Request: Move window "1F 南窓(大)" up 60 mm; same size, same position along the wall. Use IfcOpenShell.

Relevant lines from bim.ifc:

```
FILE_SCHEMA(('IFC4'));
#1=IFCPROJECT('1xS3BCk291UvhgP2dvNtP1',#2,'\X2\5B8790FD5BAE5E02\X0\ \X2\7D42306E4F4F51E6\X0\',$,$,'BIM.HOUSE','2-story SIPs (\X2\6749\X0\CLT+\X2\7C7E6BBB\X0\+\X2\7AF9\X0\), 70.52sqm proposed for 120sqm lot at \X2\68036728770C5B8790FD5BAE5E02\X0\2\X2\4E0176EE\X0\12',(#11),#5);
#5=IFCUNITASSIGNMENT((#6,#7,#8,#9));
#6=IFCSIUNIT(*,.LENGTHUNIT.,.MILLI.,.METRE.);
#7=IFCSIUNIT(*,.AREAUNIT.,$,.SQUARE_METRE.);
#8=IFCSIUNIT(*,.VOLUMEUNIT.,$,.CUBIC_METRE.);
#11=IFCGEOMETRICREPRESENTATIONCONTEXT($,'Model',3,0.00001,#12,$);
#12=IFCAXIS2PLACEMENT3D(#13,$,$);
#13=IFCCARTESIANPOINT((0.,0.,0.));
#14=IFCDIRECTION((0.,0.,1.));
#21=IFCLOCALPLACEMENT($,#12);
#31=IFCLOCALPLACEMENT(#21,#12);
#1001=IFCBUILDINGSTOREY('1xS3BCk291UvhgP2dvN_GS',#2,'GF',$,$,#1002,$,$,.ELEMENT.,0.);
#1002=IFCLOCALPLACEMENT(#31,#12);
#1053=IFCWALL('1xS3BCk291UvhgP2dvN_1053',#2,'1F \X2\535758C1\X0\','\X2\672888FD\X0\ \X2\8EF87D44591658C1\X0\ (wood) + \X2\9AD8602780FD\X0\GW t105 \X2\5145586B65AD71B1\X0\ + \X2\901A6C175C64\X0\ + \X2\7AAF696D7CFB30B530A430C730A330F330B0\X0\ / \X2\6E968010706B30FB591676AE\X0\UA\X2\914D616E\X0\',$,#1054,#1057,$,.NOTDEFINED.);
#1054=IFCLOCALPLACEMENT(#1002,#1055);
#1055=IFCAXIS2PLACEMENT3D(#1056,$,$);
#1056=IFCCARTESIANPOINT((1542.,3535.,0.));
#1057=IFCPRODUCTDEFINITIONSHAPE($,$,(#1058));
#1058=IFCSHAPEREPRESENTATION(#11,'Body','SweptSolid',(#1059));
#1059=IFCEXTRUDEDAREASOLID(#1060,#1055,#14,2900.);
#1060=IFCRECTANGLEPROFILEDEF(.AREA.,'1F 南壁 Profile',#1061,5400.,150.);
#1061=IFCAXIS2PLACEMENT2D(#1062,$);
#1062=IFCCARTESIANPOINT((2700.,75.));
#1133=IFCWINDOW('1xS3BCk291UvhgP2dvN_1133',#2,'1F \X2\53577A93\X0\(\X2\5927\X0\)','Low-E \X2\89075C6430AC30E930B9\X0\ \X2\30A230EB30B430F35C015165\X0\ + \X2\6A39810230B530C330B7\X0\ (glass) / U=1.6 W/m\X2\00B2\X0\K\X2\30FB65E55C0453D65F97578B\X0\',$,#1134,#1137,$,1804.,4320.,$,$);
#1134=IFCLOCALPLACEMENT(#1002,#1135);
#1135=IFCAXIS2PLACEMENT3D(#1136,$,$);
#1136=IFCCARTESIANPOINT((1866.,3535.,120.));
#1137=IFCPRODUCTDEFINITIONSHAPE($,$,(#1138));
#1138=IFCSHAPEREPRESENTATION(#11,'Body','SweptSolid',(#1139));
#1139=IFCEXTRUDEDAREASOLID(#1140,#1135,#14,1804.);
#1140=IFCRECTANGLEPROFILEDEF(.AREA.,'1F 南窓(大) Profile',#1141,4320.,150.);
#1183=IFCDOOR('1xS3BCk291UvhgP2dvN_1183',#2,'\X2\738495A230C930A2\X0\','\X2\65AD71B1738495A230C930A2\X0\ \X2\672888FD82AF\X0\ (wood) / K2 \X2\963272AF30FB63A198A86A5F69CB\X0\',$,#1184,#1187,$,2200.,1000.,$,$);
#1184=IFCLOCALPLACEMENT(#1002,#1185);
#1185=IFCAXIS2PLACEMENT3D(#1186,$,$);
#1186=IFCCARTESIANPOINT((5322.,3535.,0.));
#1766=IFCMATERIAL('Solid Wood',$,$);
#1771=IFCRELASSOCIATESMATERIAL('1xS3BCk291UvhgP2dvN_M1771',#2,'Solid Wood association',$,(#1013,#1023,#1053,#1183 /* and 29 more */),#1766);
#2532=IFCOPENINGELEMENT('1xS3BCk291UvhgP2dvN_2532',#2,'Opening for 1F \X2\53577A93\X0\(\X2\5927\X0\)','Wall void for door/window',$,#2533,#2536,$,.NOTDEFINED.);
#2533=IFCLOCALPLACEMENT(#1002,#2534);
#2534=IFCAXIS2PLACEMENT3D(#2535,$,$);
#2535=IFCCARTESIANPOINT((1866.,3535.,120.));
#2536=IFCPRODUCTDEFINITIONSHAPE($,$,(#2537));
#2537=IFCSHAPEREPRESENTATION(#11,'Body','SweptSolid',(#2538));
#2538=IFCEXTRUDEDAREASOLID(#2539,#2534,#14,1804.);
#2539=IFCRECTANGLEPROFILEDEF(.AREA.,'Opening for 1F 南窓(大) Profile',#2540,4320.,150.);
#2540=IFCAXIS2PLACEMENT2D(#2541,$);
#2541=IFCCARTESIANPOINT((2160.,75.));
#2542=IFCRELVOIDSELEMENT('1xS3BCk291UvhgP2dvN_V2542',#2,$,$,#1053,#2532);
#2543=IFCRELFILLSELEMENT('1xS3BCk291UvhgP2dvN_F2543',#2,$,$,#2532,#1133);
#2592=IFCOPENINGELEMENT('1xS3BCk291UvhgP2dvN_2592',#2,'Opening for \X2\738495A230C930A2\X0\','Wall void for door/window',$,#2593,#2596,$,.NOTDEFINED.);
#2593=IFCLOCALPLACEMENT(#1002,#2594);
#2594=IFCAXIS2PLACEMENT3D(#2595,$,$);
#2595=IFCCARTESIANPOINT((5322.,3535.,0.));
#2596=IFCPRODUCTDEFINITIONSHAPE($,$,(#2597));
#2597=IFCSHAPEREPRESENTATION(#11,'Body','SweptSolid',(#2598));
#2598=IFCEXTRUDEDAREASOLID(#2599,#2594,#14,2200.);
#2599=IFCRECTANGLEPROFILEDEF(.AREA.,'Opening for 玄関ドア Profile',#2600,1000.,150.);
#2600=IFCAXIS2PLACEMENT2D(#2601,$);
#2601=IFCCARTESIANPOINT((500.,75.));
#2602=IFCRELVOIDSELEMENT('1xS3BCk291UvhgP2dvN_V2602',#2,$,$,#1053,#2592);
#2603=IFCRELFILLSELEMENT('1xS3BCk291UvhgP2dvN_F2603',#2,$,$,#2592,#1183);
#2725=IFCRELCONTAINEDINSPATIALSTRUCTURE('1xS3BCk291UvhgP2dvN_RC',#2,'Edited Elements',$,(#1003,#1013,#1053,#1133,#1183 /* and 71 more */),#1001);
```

```python
import numpy as np
import ifcopenshell
import ifcopenshell.api.geometry
import ifcopenshell.util.placement
import ifcopenshell.util.unit

model = ifcopenshell.open("bim.ifc")
unit_scale = ifcopenshell.util.unit.calculate_unit_scale(model)

window = model.by_id(1133)
opening = window.FillsVoids[0].RelatingOpeningElement
dz = 0.06 / unit_scale

shift = np.array([0.0, 0.0, dz])
# The window is not placed relative to its opening, so move both.
for product in (opening, window):
    matrix = ifcopenshell.util.placement.get_local_placement(product.ObjectPlacement)
    matrix[:3, 3] += shift
    ifcopenshell.api.geometry.edit_object_placement(model, product=product, matrix=matrix, is_si=False)

print(f"moved by {dz * unit_scale:+.3f} m")

model.write("bim-out.ifc")
```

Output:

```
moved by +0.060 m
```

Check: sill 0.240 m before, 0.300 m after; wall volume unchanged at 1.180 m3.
